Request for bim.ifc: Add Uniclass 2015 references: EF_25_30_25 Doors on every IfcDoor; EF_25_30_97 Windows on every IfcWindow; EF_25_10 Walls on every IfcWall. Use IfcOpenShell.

First a look at what the model holds.

```python
import ifcopenshell

model = ifcopenshell.open("bim.ifc")
print(model.schema)
print("classifications:", [c.Name for c in model.by_type("IfcClassification")])
for ifc_class in ("IfcDoor", "IfcRoof", "IfcStair", "IfcWall", "IfcWindow"):
    print(ifc_class, len(model.by_type(ifc_class)))
```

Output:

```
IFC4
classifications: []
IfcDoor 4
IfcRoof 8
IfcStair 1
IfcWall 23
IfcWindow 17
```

```python
import ifcopenshell
import ifcopenshell.api.classification

model = ifcopenshell.open("bim.ifc")

system = ifcopenshell.api.classification.add_classification(model, classification="Uniclass 2015")

codes = {
    "IfcDoor": ("EF_25_30_25", "Doors"),
    "IfcWindow": ("EF_25_30_97", "Windows"),
    "IfcWall": ("EF_25_10", "Walls"),
}
for ifc_class, (code, name) in codes.items():
    products = model.by_type(ifc_class)
    ifcopenshell.api.classification.add_reference(
        model, products=products, classification=system, identification=code, name=name
    )
    print(code, len(products))

model.write("bim_v2.ifc")
```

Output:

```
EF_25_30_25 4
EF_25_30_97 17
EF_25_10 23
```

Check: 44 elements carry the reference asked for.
